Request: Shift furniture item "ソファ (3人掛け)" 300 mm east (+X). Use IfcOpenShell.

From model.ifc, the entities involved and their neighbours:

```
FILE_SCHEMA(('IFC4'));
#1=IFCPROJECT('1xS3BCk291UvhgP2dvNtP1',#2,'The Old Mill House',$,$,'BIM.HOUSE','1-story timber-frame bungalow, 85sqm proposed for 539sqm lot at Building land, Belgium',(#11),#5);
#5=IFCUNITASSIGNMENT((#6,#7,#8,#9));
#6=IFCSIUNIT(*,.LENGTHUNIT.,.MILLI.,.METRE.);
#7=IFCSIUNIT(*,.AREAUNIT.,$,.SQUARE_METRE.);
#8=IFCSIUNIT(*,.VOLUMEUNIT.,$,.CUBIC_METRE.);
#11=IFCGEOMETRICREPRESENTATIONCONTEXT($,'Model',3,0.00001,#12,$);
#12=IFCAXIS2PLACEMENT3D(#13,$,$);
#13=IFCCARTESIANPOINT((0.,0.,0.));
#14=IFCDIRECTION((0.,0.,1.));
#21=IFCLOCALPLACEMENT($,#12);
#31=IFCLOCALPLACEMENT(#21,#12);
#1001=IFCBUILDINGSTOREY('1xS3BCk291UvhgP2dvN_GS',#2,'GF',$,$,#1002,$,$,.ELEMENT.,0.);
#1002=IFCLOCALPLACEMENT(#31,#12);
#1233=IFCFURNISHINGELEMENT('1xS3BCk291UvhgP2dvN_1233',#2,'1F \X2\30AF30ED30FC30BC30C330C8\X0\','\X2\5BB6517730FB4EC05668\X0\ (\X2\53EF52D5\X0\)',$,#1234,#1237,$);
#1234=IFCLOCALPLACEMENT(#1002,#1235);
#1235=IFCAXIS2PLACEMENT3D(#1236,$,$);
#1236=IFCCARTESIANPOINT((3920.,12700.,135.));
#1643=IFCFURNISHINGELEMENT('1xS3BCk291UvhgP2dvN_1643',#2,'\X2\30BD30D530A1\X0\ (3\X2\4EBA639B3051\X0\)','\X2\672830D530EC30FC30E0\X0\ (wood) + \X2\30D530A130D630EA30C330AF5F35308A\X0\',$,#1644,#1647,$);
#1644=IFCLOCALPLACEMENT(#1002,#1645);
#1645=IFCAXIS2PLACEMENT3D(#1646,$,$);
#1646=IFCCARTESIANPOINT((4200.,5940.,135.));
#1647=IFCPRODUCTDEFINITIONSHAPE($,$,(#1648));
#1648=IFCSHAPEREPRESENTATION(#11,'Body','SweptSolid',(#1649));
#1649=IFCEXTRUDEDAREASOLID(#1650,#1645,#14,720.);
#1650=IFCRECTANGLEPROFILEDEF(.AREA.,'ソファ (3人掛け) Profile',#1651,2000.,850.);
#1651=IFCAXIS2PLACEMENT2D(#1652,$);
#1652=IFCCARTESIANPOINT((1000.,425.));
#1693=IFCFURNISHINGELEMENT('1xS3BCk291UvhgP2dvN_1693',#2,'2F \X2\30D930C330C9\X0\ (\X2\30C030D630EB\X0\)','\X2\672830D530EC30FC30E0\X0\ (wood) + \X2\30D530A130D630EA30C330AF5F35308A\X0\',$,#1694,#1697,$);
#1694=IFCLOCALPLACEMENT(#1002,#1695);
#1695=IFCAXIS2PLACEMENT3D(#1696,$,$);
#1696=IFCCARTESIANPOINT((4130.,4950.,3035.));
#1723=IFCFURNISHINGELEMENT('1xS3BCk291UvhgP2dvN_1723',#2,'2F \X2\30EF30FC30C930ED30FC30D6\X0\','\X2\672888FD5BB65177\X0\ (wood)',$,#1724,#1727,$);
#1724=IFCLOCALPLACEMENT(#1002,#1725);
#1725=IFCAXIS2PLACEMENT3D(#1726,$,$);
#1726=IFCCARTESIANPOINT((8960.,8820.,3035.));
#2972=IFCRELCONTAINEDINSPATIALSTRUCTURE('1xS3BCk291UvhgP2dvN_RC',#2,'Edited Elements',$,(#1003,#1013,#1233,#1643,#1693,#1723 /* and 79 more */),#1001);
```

```python
import ifcopenshell
import ifcopenshell.api.geometry
import ifcopenshell.util.placement

model = ifcopenshell.open("model.ifc")

item = model.by_guid("1xS3BCk291UvhgP2dvN_1643")
matrix = ifcopenshell.util.placement.get_local_placement(item.ObjectPlacement)
matrix[0, 3] += 300.0
ifcopenshell.api.geometry.edit_object_placement(model, product=item, matrix=matrix, is_si=False)

print(ifcopenshell.util.placement.get_local_placement(item.ObjectPlacement).round(3) + 0.0)

model.write("model_v2.ifc")
```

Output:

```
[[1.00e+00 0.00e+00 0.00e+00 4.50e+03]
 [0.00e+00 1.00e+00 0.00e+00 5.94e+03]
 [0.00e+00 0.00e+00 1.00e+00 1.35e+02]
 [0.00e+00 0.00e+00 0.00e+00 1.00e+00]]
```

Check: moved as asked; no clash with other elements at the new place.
